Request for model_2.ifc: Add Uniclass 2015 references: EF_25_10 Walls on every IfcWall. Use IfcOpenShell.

First a look at what the model holds.

```python
import ifcopenshell

model = ifcopenshell.open("model_2.ifc")
print(model.schema)
print("classifications:", [c.Name for c in model.by_type("IfcClassification")])
for ifc_class in ("IfcDoor", "IfcRoof", "IfcStair", "IfcWall", "IfcWindow"):
    print(ifc_class, len(model.by_type(ifc_class)))
```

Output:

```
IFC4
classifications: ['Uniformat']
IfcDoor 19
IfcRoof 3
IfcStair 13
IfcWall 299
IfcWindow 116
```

```python
import ifcopenshell
import ifcopenshell.api.classification

model = ifcopenshell.open("model_2.ifc")

system = ifcopenshell.api.classification.add_classification(model, classification="Uniclass 2015")

codes = {
    "IfcWall": ("EF_25_10", "Walls"),
}
for ifc_class, (code, name) in codes.items():
    products = model.by_type(ifc_class)
    ifcopenshell.api.classification.add_reference(
        model, products=products, classification=system, identification=code, name=name
    )
    print(code, len(products))

model.write("model_2_v2.ifc")
```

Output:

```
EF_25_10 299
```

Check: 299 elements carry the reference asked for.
